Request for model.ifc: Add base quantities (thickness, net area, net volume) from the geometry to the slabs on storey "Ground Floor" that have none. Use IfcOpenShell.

First a look at what the model holds.

```python
import ifcopenshell
import ifcopenshell.util.element
import ifcopenshell.util.unit

model = ifcopenshell.open("model.ifc")
print(model.schema)
for unit_type in ("LENGTHUNIT", "AREAUNIT", "VOLUMEUNIT"):
    print(unit_type, ifcopenshell.util.unit.calculate_unit_scale(model, unit_type))
storey = next(s for s in model.by_type("IfcBuildingStorey") if s.Name == "Ground Floor")
slabs = [e for e in ifcopenshell.util.element.get_decomposition(storey) if e.is_a("IfcSlab")]
for e in sorted(slabs, key=lambda e: e.id()):
    print(e.id(), e.is_a(), e.Name, list(ifcopenshell.util.element.get_psets(e, qtos_only=True)), sep=" | ")
```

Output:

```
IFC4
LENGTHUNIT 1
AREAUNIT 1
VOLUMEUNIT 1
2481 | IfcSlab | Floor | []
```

```python
import ifcopenshell
import ifcopenshell.api.pset
import ifcopenshell.geom
import ifcopenshell.util.element
import ifcopenshell.util.shape
import ifcopenshell.util.unit

model = ifcopenshell.open("model.ifc")
unit_scale = ifcopenshell.util.unit.calculate_unit_scale(model)
area_scale = ifcopenshell.util.unit.calculate_unit_scale(model, "AREAUNIT")
volume_scale = ifcopenshell.util.unit.calculate_unit_scale(model, "VOLUMEUNIT")
settings = ifcopenshell.geom.settings()

storey = next(s for s in model.by_type("IfcBuildingStorey") if s.Name == "Ground Floor")
slabs = [e for e in ifcopenshell.util.element.get_decomposition(storey) if e.is_a("IfcSlab")]

for e in sorted(slabs, key=lambda e: e.id()):
    if ifcopenshell.util.element.get_psets(e, qtos_only=True, should_inherit=False):
        continue
    # Geometry comes back in metres, in the element's own axes.
    shape = ifcopenshell.geom.create_shape(settings, e)
    values = {
        "Width": ifcopenshell.util.shape.get_z(shape.geometry) / unit_scale,
        "NetArea": ifcopenshell.util.shape.get_footprint_area(shape.geometry) / area_scale,
        "NetVolume": ifcopenshell.util.shape.get_volume(shape.geometry) / volume_scale,
    }
    qto = ifcopenshell.api.pset.add_qto(model, product=e, name="Qto_SlabBaseQuantities")
    ifcopenshell.api.pset.edit_qto(model, qto=qto, properties=values)
    print(e.id(), {k: round(v, 3) for k, v in values.items()})

model.write("model-out.ifc")
```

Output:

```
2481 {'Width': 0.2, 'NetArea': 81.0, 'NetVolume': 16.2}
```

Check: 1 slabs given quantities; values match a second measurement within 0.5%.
